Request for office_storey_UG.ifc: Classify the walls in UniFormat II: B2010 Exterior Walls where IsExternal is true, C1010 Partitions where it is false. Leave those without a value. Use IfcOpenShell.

First a look at what the model holds.

```python
import ifcopenshell
import ifcopenshell.util.element

model = ifcopenshell.open("office_storey_UG.ifc")
print(model.schema)
print("classifications:", [c.Name for c in model.by_type("IfcClassification")])
values = [ifcopenshell.util.element.get_pset(e, "Pset_WallCommon", "IsExternal") for e in model.by_type("IfcWall")]
for value in (True, False, None):
    print("IsExternal", value, values.count(value))
```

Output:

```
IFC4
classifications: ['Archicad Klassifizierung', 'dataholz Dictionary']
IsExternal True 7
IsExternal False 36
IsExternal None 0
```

```python
import ifcopenshell
import ifcopenshell.api.classification
import ifcopenshell.util.element

model = ifcopenshell.open("office_storey_UG.ifc")

system = ifcopenshell.api.classification.add_classification(model, classification="UniFormat II")

walls = model.by_type("IfcWall")
external = {e: ifcopenshell.util.element.get_pset(e, "Pset_WallCommon", "IsExternal") for e in walls}
for flag, code, name in ((True, "B2010", "Exterior Walls"), (False, "C1010", "Partitions")):
    products = [e for e in walls if external[e] is flag]
    ifcopenshell.api.classification.add_reference(
        model, products=products, classification=system, identification=code, name=name
    )
    print(code, len(products))

model.write("office_storey_UG_updated.ifc")
```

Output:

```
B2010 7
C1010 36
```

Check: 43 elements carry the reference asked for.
